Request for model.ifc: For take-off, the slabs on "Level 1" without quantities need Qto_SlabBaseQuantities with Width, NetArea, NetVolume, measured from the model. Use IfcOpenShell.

First a look at what the model holds.

```python
import ifcopenshell
import ifcopenshell.util.element
import ifcopenshell.util.unit

model = ifcopenshell.open("model.ifc")
print(model.schema)
for unit_type in ("LENGTHUNIT", "AREAUNIT", "VOLUMEUNIT"):
    print(unit_type, ifcopenshell.util.unit.calculate_unit_scale(model, unit_type))
storey = next(s for s in model.by_type("IfcBuildingStorey") if s.Name == "Level 1")
slabs = [e for e in ifcopenshell.util.element.get_decomposition(storey) if e.is_a("IfcSlab")]
for e in sorted(slabs, key=lambda e: e.id()):
    print(e.id(), e.is_a(), e.Name, list(ifcopenshell.util.element.get_psets(e, qtos_only=True)), sep=" | ")
```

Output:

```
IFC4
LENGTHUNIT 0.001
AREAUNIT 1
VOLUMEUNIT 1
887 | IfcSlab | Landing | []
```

```python
import ifcopenshell
import ifcopenshell.api.pset
import ifcopenshell.geom
import ifcopenshell.util.element
import ifcopenshell.util.shape
import ifcopenshell.util.unit

model = ifcopenshell.open("model.ifc")
unit_scale = ifcopenshell.util.unit.calculate_unit_scale(model)
area_scale = ifcopenshell.util.unit.calculate_unit_scale(model, "AREAUNIT")
volume_scale = ifcopenshell.util.unit.calculate_unit_scale(model, "VOLUMEUNIT")
settings = ifcopenshell.geom.settings()

storey = next(s for s in model.by_type("IfcBuildingStorey") if s.Name == "Level 1")
slabs = [e for e in ifcopenshell.util.element.get_decomposition(storey) if e.is_a("IfcSlab")]

for e in sorted(slabs, key=lambda e: e.id()):
    if ifcopenshell.util.element.get_psets(e, qtos_only=True, should_inherit=False):
        continue
    # Geometry comes back in metres, in the element's own axes.
    shape = ifcopenshell.geom.create_shape(settings, e)
    values = {
        "Width": ifcopenshell.util.shape.get_z(shape.geometry) / unit_scale,
        "NetArea": ifcopenshell.util.shape.get_footprint_area(shape.geometry) / area_scale,
        "NetVolume": ifcopenshell.util.shape.get_volume(shape.geometry) / volume_scale,
    }
    qto = ifcopenshell.api.pset.add_qto(model, product=e, name="Qto_SlabBaseQuantities")
    ifcopenshell.api.pset.edit_qto(model, qto=qto, properties=values)
    print(e.id(), {k: round(v, 3) for k, v in values.items()})

model.write("model-out.ifc")
```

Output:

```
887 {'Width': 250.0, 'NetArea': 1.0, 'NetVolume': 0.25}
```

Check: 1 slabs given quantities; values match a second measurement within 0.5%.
